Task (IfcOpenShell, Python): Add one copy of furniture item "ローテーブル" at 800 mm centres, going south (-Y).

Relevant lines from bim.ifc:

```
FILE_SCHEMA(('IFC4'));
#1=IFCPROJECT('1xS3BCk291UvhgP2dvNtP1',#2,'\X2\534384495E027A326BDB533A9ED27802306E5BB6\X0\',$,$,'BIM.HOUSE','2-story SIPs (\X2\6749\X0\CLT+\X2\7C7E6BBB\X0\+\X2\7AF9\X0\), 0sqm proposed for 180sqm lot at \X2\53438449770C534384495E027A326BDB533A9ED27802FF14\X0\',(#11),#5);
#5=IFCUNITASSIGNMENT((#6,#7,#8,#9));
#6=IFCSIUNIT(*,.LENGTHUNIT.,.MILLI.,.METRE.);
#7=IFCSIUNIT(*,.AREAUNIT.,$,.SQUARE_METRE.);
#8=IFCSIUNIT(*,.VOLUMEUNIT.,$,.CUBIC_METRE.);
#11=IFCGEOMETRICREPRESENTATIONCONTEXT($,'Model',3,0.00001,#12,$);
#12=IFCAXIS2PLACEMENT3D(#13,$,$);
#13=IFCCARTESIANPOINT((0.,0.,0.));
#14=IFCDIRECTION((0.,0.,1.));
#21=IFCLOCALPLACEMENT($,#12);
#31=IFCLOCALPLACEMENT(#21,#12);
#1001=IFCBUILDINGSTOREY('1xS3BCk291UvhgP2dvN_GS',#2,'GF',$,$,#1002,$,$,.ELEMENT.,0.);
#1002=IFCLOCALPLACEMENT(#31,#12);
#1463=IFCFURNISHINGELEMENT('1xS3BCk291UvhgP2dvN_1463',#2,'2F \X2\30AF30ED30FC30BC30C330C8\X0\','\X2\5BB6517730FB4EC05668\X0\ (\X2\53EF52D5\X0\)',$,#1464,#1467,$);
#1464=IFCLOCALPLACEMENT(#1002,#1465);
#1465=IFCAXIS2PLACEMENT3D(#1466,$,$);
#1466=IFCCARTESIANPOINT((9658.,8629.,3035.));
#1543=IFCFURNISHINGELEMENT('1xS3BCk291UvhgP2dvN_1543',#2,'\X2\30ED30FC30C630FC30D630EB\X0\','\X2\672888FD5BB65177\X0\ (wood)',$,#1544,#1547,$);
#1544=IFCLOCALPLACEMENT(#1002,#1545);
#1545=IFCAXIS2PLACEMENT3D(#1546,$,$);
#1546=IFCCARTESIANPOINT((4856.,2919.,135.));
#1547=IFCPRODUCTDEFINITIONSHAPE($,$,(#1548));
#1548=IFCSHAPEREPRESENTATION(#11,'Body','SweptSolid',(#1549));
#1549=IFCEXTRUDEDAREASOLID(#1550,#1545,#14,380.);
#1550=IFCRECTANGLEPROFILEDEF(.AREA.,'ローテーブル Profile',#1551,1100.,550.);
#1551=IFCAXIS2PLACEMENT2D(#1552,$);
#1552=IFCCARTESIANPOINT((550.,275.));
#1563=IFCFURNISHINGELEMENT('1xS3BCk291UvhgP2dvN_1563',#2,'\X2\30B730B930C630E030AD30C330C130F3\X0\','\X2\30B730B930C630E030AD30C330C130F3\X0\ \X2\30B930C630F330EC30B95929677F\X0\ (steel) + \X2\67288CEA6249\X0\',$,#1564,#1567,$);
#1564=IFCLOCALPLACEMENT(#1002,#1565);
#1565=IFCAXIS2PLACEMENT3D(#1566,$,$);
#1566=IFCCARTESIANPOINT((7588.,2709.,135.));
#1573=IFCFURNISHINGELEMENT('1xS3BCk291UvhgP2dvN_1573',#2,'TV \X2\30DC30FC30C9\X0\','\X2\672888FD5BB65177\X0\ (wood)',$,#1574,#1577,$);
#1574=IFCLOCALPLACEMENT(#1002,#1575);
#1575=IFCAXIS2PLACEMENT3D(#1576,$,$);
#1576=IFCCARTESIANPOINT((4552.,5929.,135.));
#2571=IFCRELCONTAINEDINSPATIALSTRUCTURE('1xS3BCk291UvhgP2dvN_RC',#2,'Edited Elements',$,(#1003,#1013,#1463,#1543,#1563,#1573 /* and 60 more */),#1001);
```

```python
import numpy as np
import ifcopenshell
import ifcopenshell.api.geometry
import ifcopenshell.api.root
import ifcopenshell.util.element
import ifcopenshell.util.placement

model = ifcopenshell.open("bim.ifc")


def reuse_history(source, copy):
    """copy_class also copies each property set's owner history, people and application; keep the originals."""
    for rel in copy.IsDefinedBy:
        if rel.is_a("IfcRelDefinesByProperties") and (history := rel.RelatingPropertyDefinition.OwnerHistory):
            rel.RelatingPropertyDefinition.OwnerHistory = source.OwnerHistory
            ifcopenshell.util.element.remove_deep2(model, history)


source = model.by_id(1543)
base = ifcopenshell.util.placement.get_local_placement(source.ObjectPlacement)
step = np.array([0.0, -1.0, 0.0]) * 800.0

for i in range(1, 2):
    copy = ifcopenshell.api.root.copy_class(model, product=source)
    copy.Representation = ifcopenshell.util.element.copy_deep(
        model, source.Representation, exclude=["IfcGeometricRepresentationContext", "IfcRepresentationMap"]
    )
    reuse_history(source, copy)
    matrix = base.copy()
    matrix[:3, 3] += i * step
    print("added at", matrix[:3, 3].round(3) + 0.0)
    ifcopenshell.api.geometry.edit_object_placement(model, product=copy, matrix=matrix, is_si=False)

model.write("bim_updated.ifc")
```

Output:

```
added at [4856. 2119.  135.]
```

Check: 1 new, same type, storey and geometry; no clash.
